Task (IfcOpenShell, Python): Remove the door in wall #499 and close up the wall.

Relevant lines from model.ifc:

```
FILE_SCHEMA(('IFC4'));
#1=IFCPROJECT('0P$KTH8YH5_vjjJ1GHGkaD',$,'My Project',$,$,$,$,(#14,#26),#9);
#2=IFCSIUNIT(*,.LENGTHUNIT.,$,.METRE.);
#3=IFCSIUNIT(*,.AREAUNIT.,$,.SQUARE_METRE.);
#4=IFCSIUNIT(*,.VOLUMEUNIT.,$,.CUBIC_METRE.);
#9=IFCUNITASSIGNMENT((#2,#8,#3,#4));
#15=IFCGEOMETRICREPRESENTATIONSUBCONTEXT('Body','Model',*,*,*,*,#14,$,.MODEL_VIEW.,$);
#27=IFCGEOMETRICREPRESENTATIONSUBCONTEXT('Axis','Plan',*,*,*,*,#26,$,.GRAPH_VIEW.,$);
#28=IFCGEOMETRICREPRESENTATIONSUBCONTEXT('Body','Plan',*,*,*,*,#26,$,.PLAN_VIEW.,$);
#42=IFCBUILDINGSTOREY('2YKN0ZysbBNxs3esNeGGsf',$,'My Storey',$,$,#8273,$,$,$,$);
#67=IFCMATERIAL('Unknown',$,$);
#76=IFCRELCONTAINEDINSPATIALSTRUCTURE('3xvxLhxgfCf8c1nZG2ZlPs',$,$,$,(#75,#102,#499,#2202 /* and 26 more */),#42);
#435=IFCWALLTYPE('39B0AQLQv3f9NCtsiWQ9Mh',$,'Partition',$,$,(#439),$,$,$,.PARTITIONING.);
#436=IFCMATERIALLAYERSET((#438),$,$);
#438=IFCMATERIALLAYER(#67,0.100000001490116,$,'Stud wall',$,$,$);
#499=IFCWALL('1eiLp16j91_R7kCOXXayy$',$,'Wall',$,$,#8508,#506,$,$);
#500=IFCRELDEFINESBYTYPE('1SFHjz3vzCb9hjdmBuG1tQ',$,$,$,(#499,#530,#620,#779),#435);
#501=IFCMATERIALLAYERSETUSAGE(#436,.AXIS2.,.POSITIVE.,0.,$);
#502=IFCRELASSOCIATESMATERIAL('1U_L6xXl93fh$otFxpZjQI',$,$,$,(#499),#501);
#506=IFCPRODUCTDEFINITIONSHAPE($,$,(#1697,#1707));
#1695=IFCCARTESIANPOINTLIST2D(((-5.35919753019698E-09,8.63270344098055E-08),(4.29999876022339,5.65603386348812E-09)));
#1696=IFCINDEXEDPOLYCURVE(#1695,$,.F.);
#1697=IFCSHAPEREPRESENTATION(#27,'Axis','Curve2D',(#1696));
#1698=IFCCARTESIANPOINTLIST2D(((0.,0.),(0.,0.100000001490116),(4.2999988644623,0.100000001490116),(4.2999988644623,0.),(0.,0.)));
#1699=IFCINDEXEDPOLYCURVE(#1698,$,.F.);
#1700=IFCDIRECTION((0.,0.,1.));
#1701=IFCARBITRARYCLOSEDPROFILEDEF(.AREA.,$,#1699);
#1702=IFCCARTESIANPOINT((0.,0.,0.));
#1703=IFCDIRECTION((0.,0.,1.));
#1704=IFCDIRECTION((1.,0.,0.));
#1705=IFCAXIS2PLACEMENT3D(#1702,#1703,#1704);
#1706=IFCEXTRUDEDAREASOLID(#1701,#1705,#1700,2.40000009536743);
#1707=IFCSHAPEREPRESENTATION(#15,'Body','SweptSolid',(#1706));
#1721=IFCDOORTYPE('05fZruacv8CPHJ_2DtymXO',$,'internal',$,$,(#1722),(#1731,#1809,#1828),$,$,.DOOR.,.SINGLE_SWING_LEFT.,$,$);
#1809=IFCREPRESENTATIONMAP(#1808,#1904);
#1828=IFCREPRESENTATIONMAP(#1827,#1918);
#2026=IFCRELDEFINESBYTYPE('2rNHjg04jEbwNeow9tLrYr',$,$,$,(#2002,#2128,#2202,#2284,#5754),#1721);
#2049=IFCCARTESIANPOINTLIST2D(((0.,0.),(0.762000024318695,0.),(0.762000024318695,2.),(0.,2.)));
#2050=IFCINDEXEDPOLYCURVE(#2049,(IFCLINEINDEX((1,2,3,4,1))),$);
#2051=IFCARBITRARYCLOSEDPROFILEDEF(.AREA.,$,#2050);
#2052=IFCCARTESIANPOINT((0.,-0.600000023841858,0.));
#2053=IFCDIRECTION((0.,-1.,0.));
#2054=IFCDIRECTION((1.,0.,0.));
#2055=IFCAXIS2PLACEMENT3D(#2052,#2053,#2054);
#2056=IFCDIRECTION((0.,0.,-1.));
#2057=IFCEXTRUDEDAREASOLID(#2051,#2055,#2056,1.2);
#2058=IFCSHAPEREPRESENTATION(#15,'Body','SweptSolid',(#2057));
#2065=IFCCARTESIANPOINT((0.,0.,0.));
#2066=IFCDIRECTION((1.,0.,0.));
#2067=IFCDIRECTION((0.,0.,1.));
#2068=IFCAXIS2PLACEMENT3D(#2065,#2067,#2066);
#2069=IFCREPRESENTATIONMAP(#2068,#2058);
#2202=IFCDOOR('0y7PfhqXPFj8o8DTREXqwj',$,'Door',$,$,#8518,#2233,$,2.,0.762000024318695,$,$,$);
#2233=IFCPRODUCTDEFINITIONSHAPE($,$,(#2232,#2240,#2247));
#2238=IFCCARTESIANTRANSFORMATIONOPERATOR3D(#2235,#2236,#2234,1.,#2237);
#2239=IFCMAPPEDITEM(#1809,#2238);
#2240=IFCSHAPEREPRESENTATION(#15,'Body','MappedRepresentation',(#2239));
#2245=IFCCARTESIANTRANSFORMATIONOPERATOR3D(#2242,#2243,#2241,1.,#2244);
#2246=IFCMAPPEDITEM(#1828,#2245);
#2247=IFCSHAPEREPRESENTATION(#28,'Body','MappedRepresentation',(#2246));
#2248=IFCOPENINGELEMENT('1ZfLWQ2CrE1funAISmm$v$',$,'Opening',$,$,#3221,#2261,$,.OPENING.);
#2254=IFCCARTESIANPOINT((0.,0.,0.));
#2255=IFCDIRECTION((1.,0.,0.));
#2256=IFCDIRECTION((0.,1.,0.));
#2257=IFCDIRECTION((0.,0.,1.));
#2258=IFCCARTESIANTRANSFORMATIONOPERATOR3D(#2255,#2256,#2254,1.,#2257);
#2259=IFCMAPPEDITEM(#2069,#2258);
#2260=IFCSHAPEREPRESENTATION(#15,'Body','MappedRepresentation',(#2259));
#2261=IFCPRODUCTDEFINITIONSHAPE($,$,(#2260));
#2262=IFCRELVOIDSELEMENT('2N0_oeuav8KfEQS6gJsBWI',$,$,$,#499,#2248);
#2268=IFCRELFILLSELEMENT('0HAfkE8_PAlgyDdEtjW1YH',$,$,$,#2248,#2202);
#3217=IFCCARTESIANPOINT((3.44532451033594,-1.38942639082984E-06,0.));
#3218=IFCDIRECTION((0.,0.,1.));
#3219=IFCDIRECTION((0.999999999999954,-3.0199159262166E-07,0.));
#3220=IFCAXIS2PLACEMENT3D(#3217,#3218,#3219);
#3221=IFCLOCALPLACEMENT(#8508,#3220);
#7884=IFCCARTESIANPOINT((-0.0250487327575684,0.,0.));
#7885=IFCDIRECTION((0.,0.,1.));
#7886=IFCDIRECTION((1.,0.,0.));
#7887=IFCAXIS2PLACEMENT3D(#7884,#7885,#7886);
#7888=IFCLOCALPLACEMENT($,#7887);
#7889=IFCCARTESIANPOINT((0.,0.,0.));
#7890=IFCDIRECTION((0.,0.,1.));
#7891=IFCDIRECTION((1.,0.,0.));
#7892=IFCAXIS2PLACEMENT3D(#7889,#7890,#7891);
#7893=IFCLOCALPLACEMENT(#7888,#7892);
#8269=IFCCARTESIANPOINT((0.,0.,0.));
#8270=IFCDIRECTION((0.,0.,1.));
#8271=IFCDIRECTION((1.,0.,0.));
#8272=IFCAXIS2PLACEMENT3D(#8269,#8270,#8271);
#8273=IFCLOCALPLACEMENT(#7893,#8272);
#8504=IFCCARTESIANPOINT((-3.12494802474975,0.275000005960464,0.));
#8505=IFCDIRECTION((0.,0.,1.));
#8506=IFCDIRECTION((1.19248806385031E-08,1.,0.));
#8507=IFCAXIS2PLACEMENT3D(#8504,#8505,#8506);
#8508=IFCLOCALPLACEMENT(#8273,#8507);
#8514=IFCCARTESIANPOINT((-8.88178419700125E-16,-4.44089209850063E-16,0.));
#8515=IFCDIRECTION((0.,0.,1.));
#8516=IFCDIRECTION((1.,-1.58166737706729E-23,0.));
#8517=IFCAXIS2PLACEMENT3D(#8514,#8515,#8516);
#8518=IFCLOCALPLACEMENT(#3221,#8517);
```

```python
import ifcopenshell
import ifcopenshell.api.feature
import ifcopenshell.api.root
import ifcopenshell.geom
import ifcopenshell.util.shape

model = ifcopenshell.open("model.ifc")
settings = ifcopenshell.geom.settings()


def volume(element):
    """Net volume in cubic metres, openings subtracted."""
    shape = ifcopenshell.geom.create_shape(settings, element)
    return ifcopenshell.util.shape.get_volume(shape.geometry)


door = model.by_guid("0y7PfhqXPFj8o8DTREXqwj")
opening = door.FillsVoids[0].RelatingOpeningElement
wall = opening.VoidsElements[0].RelatingBuildingElement
before = volume(wall)

ifcopenshell.api.root.remove_product(model, product=door)
ifcopenshell.api.feature.remove_feature(model, feature=opening)

after = volume(wall)

print(f"wall volume {before:.3f} -> {after:.3f} m3")

model.write("model_edited.ifc")
```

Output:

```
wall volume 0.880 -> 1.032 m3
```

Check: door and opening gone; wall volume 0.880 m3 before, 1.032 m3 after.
